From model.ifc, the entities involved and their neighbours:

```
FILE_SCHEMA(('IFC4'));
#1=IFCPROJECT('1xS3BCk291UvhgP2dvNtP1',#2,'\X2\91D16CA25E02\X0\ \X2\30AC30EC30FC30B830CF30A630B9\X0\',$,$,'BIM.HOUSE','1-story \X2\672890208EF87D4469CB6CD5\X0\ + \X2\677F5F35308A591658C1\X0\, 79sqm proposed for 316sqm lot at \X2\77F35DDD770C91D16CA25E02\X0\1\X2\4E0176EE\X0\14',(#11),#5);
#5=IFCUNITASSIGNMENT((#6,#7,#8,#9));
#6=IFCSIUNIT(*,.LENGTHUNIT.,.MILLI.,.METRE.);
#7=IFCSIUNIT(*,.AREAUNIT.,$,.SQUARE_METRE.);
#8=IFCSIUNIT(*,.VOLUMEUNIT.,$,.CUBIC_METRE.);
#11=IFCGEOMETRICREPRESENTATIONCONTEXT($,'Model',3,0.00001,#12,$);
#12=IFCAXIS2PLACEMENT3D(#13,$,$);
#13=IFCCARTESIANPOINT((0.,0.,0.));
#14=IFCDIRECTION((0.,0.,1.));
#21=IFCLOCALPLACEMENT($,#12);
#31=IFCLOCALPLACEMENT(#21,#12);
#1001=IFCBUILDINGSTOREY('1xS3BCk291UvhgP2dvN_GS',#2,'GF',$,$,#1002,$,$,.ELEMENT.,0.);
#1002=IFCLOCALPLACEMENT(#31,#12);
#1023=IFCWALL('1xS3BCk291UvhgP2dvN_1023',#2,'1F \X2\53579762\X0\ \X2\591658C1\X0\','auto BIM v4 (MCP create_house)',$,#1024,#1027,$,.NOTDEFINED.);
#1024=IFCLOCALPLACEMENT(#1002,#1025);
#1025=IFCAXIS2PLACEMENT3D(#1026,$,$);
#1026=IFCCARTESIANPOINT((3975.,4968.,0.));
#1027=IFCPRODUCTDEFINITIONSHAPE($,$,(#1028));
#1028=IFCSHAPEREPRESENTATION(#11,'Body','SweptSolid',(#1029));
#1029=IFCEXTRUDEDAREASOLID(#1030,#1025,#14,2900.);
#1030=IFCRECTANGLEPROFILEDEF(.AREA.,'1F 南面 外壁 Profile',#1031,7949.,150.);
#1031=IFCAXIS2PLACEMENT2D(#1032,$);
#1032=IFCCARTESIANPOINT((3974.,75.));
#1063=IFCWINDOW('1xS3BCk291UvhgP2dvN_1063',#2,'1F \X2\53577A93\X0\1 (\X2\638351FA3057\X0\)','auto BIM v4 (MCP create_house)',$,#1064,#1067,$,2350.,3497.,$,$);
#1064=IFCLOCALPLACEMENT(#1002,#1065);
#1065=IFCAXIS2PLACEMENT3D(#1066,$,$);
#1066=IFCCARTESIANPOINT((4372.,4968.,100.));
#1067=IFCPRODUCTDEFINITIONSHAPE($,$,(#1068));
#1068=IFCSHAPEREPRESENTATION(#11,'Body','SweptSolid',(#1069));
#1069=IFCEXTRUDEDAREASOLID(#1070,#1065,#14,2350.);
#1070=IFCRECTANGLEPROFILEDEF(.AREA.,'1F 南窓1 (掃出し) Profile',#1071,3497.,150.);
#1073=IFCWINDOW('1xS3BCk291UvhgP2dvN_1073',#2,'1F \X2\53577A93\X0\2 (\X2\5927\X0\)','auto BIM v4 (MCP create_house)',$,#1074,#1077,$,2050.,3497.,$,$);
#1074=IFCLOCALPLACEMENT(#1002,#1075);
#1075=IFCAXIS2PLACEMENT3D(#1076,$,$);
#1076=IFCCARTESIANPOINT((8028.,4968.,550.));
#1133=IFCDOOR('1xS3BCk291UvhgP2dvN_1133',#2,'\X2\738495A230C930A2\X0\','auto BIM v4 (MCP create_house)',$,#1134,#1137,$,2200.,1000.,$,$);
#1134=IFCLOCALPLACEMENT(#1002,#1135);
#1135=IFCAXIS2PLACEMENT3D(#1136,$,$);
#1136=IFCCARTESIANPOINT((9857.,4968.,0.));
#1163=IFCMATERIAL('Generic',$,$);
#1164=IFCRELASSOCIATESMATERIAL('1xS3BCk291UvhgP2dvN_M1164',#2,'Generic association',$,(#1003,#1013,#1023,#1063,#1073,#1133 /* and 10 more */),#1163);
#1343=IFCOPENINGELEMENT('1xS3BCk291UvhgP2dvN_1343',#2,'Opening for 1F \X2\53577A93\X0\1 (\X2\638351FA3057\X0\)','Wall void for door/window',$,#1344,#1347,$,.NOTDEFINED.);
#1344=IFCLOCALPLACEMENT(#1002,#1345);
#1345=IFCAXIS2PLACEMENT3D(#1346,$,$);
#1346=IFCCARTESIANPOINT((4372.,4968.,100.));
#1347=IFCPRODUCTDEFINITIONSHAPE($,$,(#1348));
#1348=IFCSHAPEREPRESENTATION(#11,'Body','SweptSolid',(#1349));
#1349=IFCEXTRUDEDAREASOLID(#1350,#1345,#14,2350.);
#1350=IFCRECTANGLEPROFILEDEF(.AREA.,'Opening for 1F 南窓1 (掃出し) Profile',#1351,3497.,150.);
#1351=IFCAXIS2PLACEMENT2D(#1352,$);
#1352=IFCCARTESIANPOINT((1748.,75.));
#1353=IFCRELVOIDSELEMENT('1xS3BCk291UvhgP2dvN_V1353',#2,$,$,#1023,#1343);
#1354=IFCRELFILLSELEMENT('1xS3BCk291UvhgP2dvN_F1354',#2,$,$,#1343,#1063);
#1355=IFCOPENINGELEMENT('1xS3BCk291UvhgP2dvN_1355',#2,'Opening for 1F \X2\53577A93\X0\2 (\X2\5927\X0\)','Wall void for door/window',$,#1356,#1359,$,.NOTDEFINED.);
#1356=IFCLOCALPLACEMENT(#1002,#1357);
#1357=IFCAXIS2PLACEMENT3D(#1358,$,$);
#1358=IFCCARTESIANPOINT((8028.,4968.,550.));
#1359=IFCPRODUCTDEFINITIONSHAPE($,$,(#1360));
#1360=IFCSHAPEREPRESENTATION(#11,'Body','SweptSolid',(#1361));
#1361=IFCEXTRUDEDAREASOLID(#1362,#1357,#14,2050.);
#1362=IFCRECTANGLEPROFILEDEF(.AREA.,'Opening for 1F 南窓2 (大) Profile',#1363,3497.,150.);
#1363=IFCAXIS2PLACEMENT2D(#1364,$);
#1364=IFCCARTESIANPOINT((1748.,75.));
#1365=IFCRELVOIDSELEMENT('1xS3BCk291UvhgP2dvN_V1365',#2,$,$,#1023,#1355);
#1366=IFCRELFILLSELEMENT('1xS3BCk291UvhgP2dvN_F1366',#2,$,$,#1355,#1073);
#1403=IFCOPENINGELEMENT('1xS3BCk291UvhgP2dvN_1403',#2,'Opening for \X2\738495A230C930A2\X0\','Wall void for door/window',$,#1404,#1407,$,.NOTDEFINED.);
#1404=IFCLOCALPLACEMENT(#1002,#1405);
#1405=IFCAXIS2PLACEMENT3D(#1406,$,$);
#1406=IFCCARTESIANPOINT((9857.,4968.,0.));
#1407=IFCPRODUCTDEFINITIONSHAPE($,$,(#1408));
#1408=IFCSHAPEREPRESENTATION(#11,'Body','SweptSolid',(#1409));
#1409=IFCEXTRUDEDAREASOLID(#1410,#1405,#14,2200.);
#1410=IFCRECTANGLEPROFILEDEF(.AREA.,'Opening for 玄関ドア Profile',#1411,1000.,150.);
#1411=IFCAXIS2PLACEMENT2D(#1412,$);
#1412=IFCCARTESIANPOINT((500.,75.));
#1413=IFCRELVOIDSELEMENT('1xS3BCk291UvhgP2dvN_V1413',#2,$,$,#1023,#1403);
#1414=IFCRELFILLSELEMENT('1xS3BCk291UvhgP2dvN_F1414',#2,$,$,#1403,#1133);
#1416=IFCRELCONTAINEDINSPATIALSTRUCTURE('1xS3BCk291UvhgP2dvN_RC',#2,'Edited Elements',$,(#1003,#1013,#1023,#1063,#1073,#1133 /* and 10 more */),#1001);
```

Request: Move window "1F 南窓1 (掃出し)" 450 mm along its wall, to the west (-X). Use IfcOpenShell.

```python
import ifcopenshell
import ifcopenshell.api.geometry
import ifcopenshell.util.placement
import ifcopenshell.util.unit

model = ifcopenshell.open("model.ifc")
unit_scale = ifcopenshell.util.unit.calculate_unit_scale(model)

window = model.by_id(1063)
opening = window.FillsVoids[0].RelatingOpeningElement
wall = opening.VoidsElements[0].RelatingBuildingElement

wall_matrix = ifcopenshell.util.placement.get_local_placement(wall.ObjectPlacement)
shift = wall_matrix[:3, 0] * -0.45 / unit_scale
before = ifcopenshell.util.placement.get_local_placement(window.ObjectPlacement)[:3, 3].copy()

# The window is not placed relative to its opening, so move both.
for product in (opening, window):
    matrix = ifcopenshell.util.placement.get_local_placement(product.ObjectPlacement)
    matrix[:3, 3] += shift
    ifcopenshell.api.geometry.edit_object_placement(model, product=product, matrix=matrix, is_si=False)

after = ifcopenshell.util.placement.get_local_placement(window.ObjectPlacement)[:3, 3]
print("window moved by", (after - before).round(3) + 0.0)

model.write("model_v2.ifc")
```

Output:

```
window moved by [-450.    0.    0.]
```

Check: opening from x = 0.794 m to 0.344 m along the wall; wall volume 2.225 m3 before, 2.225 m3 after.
